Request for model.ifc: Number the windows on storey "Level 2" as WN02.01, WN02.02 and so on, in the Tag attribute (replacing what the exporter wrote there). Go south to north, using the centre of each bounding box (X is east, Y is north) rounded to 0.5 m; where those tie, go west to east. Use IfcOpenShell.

First a look at what the model holds.

```python
import ifcopenshell
import ifcopenshell.util.element
import ifcopenshell.util.placement

model = ifcopenshell.open("model.ifc")
print(model.schema)
storey = next(s for s in model.by_type("IfcBuildingStorey") if s.Name == "Level 2")
windows = [e for e in ifcopenshell.util.element.get_decomposition(storey) if e.is_a("IfcWindow")]
for e in sorted(windows, key=lambda e: e.id()):
    origin = ifcopenshell.util.placement.get_local_placement(e.ObjectPlacement)[:3, 3]
    print(e.id(), e.Tag, e.Name, origin.round(2) + 0.0, sep=" | ")
```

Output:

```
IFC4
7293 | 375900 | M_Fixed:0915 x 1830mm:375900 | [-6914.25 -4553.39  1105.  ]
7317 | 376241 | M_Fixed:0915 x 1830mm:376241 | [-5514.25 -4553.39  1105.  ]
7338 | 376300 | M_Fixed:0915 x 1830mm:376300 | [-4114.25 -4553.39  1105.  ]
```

```python
import ifcopenshell
import ifcopenshell.geom
import ifcopenshell.util.element
import ifcopenshell.util.shape

model = ifcopenshell.open("model.ifc")
settings = ifcopenshell.geom.settings()
settings.set("use-world-coords", True)


def centre(element):
    shape = ifcopenshell.geom.create_shape(settings, element)
    return ifcopenshell.util.shape.get_bbox_centroid(shape.geometry)


storey = next(s for s in model.by_type("IfcBuildingStorey") if s.Name == "Level 2")
windows = [e for e in ifcopenshell.util.element.get_decomposition(storey) if e.is_a("IfcWindow")]

# Insertion points can sit at a corner or the storey origin, so sort by the geometry (in metres).
centres = {e: centre(e) for e in windows}
windows.sort(key=lambda e: (round(centres[e][1] / 0.5), centres[e][0]))

for i, e in enumerate(windows, start=1):
    number = f"WN02.{i:02d}"
    e.Tag = number
    print(e.id(), number)

model.write("model_updated.ifc")
```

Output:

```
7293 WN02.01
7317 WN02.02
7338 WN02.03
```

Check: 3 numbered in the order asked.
